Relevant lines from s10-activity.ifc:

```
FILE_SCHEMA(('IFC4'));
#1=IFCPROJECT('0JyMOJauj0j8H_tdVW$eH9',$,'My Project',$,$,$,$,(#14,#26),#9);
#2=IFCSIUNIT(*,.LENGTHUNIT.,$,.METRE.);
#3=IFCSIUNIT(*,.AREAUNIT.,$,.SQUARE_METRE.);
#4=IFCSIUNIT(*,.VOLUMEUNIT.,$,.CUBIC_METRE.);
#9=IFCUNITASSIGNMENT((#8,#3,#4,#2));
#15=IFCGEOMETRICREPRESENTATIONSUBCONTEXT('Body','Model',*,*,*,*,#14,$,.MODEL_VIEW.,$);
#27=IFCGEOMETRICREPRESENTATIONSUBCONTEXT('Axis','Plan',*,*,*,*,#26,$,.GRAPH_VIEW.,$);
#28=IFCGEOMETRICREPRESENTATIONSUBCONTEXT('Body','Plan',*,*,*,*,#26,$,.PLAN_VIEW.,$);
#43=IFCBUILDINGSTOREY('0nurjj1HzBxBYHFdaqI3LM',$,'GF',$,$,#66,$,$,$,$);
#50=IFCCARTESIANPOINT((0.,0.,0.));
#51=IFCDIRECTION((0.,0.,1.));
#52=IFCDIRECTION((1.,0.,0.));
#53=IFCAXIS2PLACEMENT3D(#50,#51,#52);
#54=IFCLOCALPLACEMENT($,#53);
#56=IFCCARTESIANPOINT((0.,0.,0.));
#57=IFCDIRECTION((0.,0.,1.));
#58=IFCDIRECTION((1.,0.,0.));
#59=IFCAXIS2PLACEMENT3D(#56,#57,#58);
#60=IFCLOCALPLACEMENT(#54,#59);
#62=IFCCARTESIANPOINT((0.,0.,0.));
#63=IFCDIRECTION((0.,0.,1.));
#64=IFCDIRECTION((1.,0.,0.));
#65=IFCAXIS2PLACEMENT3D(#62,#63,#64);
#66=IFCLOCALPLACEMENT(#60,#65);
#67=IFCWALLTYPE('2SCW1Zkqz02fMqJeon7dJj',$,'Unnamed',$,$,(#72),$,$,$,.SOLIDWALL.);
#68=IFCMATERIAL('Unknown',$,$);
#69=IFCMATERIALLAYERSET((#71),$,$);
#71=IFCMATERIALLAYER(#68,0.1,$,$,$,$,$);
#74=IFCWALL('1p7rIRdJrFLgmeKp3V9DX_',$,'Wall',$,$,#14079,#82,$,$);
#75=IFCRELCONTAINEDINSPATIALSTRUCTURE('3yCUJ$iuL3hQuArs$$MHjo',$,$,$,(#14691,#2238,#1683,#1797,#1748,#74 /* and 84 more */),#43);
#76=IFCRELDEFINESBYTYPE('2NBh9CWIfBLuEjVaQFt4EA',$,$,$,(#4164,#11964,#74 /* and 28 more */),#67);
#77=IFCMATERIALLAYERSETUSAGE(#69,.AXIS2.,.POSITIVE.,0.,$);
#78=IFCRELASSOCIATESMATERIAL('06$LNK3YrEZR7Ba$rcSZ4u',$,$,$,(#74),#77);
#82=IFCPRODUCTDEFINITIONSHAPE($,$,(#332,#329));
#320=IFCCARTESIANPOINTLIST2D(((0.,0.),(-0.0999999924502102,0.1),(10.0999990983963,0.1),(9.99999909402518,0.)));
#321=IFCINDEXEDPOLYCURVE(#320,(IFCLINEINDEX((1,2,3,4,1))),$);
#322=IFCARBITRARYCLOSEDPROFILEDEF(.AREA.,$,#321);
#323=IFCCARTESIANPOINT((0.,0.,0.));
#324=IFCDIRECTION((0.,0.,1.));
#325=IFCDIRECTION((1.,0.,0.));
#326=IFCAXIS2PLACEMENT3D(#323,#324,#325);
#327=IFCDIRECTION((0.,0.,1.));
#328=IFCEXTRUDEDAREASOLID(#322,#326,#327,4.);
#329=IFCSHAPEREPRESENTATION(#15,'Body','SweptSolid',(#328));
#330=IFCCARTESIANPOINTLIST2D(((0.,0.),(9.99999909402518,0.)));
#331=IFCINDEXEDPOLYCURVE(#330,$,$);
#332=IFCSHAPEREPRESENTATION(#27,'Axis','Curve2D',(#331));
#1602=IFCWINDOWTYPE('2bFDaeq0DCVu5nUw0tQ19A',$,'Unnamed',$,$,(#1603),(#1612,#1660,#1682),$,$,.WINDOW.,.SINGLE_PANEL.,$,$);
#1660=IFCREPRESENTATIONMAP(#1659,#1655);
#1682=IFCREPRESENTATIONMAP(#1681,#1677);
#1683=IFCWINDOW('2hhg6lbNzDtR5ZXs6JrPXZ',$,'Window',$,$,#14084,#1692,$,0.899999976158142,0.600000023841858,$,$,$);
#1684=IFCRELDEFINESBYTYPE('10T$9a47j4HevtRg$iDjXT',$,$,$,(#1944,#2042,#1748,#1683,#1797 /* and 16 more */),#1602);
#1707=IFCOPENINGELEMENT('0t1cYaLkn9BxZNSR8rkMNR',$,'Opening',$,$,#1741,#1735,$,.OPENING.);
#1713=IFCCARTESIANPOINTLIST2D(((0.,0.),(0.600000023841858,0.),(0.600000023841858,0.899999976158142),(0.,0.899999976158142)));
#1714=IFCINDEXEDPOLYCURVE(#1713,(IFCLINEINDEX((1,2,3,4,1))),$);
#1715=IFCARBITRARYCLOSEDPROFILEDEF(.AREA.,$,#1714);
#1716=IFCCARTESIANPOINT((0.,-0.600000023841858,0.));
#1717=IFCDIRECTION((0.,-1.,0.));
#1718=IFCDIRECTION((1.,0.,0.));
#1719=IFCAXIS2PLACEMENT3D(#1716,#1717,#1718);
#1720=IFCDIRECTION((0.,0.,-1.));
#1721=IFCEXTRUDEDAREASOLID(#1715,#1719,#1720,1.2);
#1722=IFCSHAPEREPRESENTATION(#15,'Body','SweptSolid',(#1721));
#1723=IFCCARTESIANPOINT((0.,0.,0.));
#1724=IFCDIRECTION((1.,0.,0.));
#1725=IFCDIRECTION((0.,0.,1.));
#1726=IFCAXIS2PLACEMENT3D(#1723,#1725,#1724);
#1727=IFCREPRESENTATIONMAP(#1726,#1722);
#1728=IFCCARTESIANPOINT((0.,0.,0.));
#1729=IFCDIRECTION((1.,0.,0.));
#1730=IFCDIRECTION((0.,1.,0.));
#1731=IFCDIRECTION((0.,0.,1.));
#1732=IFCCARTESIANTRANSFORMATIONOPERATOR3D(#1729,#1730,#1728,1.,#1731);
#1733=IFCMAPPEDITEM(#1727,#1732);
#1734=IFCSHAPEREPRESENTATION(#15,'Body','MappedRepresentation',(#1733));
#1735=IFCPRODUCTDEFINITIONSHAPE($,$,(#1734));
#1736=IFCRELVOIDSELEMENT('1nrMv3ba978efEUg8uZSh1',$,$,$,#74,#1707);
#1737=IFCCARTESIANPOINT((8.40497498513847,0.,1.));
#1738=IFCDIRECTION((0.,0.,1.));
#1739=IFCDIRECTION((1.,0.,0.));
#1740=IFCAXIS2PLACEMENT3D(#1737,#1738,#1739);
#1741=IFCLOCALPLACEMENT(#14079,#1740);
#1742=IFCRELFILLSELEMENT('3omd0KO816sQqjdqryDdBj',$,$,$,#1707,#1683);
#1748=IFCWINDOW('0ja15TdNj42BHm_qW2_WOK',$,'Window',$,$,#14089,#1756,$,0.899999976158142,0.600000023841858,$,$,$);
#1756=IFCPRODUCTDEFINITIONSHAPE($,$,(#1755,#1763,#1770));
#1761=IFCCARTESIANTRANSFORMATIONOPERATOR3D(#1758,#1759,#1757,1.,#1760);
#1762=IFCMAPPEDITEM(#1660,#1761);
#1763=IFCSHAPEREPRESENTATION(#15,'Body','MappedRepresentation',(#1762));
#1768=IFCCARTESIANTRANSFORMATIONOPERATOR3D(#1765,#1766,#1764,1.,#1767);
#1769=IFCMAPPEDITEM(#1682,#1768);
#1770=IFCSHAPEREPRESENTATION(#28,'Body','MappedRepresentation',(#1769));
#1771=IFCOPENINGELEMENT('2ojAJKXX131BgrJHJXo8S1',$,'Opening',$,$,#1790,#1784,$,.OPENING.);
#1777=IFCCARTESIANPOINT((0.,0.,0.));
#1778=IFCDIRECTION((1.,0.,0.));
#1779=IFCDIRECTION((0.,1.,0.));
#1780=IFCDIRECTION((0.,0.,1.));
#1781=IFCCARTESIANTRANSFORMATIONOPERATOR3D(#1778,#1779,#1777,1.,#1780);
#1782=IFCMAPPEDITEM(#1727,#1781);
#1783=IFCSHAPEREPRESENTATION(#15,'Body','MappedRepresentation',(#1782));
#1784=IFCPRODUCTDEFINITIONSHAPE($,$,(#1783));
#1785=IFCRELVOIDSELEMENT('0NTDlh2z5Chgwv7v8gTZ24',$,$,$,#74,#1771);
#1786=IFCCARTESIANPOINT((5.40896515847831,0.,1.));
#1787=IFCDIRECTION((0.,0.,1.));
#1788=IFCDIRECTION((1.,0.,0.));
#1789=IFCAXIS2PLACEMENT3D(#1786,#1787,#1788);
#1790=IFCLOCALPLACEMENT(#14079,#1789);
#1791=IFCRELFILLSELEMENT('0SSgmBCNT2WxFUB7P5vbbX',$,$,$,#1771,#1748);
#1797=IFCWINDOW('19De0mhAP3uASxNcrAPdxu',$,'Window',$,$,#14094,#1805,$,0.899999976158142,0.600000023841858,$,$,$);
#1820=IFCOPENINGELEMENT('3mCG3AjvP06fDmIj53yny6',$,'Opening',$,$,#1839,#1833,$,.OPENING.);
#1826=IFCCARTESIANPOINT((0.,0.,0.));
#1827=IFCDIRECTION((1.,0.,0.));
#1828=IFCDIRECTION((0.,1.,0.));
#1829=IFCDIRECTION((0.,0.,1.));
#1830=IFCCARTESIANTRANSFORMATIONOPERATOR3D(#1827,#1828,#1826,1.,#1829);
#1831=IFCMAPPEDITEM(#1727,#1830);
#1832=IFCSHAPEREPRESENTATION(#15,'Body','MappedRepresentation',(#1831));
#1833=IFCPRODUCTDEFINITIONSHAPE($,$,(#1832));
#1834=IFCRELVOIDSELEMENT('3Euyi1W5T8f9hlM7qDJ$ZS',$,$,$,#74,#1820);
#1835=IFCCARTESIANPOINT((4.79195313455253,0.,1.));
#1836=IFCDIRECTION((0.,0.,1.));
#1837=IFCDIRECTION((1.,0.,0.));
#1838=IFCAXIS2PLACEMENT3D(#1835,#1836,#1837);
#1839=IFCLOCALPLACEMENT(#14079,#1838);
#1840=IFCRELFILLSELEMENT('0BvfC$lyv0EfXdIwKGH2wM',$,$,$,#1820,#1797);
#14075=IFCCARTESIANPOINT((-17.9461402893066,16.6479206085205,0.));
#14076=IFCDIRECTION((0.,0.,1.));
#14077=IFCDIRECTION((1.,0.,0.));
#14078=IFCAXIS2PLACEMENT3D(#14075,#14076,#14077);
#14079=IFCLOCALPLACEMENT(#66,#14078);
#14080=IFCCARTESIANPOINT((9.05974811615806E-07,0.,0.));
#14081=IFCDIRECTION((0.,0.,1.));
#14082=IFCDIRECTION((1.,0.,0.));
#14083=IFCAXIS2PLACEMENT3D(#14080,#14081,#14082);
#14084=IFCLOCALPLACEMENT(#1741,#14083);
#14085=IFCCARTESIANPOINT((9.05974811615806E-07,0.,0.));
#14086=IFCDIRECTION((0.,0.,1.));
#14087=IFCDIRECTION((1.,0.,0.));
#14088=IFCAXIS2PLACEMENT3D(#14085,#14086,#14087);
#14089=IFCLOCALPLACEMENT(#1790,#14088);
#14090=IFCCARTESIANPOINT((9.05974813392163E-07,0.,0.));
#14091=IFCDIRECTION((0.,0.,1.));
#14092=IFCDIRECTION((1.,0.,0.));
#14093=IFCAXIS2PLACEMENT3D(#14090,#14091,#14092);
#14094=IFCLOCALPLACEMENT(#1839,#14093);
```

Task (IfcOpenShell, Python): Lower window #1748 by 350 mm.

```python
import numpy as np
import ifcopenshell
import ifcopenshell.api.geometry
import ifcopenshell.util.placement
import ifcopenshell.util.unit

model = ifcopenshell.open("s10-activity.ifc")
unit_scale = ifcopenshell.util.unit.calculate_unit_scale(model)

window = model.by_id(1748)
opening = window.FillsVoids[0].RelatingOpeningElement
dz = -0.35

shift = np.array([0.0, 0.0, dz])
# The window is placed relative to its opening, so it follows when the opening moves.
matrix = ifcopenshell.util.placement.get_local_placement(opening.ObjectPlacement)
matrix[:3, 3] += shift
ifcopenshell.api.geometry.edit_object_placement(
    model, product=opening, matrix=matrix, is_si=False, should_transform_children=True
)

print(f"moved by {dz * unit_scale:+.3f} m")

model.write("s10-activity_rev.ifc")
```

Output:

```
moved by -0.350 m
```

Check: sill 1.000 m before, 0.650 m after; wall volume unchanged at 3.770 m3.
